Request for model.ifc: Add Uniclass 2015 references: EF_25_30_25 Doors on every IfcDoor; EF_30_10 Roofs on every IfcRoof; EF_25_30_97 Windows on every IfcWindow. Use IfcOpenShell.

First a look at what the model holds.

```python
import ifcopenshell

model = ifcopenshell.open("model.ifc")
print(model.schema)
print("classifications:", [c.Name for c in model.by_type("IfcClassification")])
for ifc_class in ("IfcDoor", "IfcRoof", "IfcStair", "IfcWall", "IfcWindow"):
    print(ifc_class, len(model.by_type(ifc_class)))
```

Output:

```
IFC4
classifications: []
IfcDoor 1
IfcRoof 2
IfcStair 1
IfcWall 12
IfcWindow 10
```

```python
import ifcopenshell
import ifcopenshell.api.classification

model = ifcopenshell.open("model.ifc")

system = ifcopenshell.api.classification.add_classification(model, classification="Uniclass 2015")

codes = {
    "IfcDoor": ("EF_25_30_25", "Doors"),
    "IfcRoof": ("EF_30_10", "Roofs"),
    "IfcWindow": ("EF_25_30_97", "Windows"),
}
for ifc_class, (code, name) in codes.items():
    products = model.by_type(ifc_class)
    ifcopenshell.api.classification.add_reference(
        model, products=products, classification=system, identification=code, name=name
    )
    print(code, len(products))

model.write("model_v2.ifc")
```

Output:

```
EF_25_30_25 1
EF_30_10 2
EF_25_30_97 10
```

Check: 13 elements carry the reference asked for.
